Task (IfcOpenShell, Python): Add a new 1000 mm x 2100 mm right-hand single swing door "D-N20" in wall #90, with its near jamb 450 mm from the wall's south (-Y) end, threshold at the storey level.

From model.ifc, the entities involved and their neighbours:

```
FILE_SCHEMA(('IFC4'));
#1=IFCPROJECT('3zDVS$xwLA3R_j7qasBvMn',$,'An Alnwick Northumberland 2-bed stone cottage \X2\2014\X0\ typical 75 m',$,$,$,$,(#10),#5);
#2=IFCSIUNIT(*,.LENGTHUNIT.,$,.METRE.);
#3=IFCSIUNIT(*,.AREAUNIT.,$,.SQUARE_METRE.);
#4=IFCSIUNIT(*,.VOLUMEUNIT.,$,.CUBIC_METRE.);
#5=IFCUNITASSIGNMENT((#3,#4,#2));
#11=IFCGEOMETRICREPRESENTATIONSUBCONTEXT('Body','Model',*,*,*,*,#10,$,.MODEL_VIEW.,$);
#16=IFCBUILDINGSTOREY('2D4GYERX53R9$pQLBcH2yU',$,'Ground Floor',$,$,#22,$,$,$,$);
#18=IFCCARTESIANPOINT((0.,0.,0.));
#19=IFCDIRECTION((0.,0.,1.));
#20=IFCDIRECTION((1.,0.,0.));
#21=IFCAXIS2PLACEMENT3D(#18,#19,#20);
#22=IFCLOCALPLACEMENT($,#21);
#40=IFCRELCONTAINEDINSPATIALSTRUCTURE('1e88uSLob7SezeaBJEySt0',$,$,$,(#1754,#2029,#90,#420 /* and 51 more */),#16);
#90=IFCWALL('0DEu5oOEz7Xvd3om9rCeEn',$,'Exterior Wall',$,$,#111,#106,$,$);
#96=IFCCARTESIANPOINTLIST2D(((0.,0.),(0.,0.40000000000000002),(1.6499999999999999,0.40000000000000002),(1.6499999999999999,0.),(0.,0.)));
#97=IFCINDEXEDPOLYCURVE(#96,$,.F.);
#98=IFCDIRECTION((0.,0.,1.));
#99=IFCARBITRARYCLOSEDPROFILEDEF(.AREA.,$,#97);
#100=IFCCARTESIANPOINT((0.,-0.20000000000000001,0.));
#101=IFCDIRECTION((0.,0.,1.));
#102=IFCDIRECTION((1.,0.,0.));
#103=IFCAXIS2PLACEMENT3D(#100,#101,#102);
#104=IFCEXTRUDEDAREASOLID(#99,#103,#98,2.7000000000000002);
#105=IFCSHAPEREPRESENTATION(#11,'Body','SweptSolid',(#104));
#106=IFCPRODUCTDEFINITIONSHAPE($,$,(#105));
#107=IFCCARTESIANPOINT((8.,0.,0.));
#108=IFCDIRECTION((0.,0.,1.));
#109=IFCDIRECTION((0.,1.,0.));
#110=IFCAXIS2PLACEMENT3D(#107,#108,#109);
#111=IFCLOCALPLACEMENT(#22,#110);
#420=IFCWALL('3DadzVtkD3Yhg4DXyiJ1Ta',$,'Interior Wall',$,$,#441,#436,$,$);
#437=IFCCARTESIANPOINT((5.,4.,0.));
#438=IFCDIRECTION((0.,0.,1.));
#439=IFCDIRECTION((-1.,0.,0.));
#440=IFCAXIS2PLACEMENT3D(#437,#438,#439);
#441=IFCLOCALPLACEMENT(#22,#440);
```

```python
import numpy as np
import ifcopenshell
import ifcopenshell.api.feature
import ifcopenshell.api.geometry
import ifcopenshell.api.root
import ifcopenshell.api.spatial
import ifcopenshell.geom
import ifcopenshell.util.element
import ifcopenshell.util.placement
import ifcopenshell.util.representation
import ifcopenshell.util.shape
import ifcopenshell.util.unit

model = ifcopenshell.open("model.ifc")
unit_scale = ifcopenshell.util.unit.calculate_unit_scale(model)
settings = ifcopenshell.geom.settings()


def volume(element):
    """Net volume in cubic metres, openings subtracted."""
    shape = ifcopenshell.geom.create_shape(settings, element)
    return ifcopenshell.util.shape.get_volume(shape.geometry)


wall = model.by_guid("0DEu5oOEz7Xvd3om9rCeEn")
storey = ifcopenshell.util.element.get_container(wall, ifc_class="IfcBuildingStorey")
context = ifcopenshell.util.representation.get_context(model, "Model", "Body", "MODEL_VIEW")
before = volume(wall)

width, height, from_end, sill = 1, 2.1, 0.45, 0.0  # metres

# The wall runs along its own X axis, and the end named is its -X end.
wall_shape = ifcopenshell.geom.create_shape(settings, wall)
x, y, z = ifcopenshell.util.shape.get_vertices(wall_shape.geometry).T
start = x.min() + from_end
face, thickness = float(y.min()), float(y.max() - y.min())
wall_matrix = ifcopenshell.util.placement.get_local_placement(wall.ObjectPlacement)
level = ifcopenshell.util.placement.get_local_placement(storey.ObjectPlacement)[2, 3]


def in_wall(x, y):
    """Placement at x, y metres in the wall's axes, at sill height."""
    matrix = wall_matrix.copy()
    matrix[:, 3] = wall_matrix @ np.array([x / unit_scale, y / unit_scale, 0.0, 1.0])
    matrix[2, 3] = level + sill / unit_scale
    return matrix


# Opening: a box that overshoots both wall faces by 50 mm.
opening = ifcopenshell.api.root.create_entity(model, ifc_class="IfcOpeningElement", predefined_type="OPENING")
box = ifcopenshell.api.geometry.add_wall_representation(
    model, context=context, length=width, height=height, thickness=thickness + 0.1
)
ifcopenshell.api.geometry.assign_representation(model, product=opening, representation=box)
ifcopenshell.api.geometry.edit_object_placement(model, product=opening, matrix=in_wall(start, face - 0.05), is_si=False)
ifcopenshell.api.feature.add_feature(model, feature=opening, element=wall)

door = ifcopenshell.api.root.create_entity(model, ifc_class="IfcDoor", name="D-N20", predefined_type="DOOR")
door.OverallWidth, door.OverallHeight = width / unit_scale, height / unit_scale
door.OperationType = "SINGLE_SWING_RIGHT"
body = ifcopenshell.api.geometry.add_door_representation(
    model,
    context=context,
    overall_width=door.OverallWidth,
    overall_height=door.OverallHeight,
    operation_type="SINGLE_SWING_RIGHT",
    lining_properties={"LiningDepth": thickness / unit_scale, "ThresholdDepth": thickness / unit_scale},
)
ifcopenshell.api.geometry.assign_representation(model, product=door, representation=body)
ifcopenshell.api.spatial.assign_container(model, products=[door], relating_structure=storey)
ifcopenshell.api.feature.add_filling(model, opening=opening, element=door)

# The lining spans the wall, so the door starts at the wall face.
ifcopenshell.api.geometry.edit_object_placement(model, product=door, matrix=in_wall(start, face), is_si=False)

after = volume(wall)

print(f"wall volume {before:.3f} -> {after:.3f} m3")

model.write("model_updated.ifc")
```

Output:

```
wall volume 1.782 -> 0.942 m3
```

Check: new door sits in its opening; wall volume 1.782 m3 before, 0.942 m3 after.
